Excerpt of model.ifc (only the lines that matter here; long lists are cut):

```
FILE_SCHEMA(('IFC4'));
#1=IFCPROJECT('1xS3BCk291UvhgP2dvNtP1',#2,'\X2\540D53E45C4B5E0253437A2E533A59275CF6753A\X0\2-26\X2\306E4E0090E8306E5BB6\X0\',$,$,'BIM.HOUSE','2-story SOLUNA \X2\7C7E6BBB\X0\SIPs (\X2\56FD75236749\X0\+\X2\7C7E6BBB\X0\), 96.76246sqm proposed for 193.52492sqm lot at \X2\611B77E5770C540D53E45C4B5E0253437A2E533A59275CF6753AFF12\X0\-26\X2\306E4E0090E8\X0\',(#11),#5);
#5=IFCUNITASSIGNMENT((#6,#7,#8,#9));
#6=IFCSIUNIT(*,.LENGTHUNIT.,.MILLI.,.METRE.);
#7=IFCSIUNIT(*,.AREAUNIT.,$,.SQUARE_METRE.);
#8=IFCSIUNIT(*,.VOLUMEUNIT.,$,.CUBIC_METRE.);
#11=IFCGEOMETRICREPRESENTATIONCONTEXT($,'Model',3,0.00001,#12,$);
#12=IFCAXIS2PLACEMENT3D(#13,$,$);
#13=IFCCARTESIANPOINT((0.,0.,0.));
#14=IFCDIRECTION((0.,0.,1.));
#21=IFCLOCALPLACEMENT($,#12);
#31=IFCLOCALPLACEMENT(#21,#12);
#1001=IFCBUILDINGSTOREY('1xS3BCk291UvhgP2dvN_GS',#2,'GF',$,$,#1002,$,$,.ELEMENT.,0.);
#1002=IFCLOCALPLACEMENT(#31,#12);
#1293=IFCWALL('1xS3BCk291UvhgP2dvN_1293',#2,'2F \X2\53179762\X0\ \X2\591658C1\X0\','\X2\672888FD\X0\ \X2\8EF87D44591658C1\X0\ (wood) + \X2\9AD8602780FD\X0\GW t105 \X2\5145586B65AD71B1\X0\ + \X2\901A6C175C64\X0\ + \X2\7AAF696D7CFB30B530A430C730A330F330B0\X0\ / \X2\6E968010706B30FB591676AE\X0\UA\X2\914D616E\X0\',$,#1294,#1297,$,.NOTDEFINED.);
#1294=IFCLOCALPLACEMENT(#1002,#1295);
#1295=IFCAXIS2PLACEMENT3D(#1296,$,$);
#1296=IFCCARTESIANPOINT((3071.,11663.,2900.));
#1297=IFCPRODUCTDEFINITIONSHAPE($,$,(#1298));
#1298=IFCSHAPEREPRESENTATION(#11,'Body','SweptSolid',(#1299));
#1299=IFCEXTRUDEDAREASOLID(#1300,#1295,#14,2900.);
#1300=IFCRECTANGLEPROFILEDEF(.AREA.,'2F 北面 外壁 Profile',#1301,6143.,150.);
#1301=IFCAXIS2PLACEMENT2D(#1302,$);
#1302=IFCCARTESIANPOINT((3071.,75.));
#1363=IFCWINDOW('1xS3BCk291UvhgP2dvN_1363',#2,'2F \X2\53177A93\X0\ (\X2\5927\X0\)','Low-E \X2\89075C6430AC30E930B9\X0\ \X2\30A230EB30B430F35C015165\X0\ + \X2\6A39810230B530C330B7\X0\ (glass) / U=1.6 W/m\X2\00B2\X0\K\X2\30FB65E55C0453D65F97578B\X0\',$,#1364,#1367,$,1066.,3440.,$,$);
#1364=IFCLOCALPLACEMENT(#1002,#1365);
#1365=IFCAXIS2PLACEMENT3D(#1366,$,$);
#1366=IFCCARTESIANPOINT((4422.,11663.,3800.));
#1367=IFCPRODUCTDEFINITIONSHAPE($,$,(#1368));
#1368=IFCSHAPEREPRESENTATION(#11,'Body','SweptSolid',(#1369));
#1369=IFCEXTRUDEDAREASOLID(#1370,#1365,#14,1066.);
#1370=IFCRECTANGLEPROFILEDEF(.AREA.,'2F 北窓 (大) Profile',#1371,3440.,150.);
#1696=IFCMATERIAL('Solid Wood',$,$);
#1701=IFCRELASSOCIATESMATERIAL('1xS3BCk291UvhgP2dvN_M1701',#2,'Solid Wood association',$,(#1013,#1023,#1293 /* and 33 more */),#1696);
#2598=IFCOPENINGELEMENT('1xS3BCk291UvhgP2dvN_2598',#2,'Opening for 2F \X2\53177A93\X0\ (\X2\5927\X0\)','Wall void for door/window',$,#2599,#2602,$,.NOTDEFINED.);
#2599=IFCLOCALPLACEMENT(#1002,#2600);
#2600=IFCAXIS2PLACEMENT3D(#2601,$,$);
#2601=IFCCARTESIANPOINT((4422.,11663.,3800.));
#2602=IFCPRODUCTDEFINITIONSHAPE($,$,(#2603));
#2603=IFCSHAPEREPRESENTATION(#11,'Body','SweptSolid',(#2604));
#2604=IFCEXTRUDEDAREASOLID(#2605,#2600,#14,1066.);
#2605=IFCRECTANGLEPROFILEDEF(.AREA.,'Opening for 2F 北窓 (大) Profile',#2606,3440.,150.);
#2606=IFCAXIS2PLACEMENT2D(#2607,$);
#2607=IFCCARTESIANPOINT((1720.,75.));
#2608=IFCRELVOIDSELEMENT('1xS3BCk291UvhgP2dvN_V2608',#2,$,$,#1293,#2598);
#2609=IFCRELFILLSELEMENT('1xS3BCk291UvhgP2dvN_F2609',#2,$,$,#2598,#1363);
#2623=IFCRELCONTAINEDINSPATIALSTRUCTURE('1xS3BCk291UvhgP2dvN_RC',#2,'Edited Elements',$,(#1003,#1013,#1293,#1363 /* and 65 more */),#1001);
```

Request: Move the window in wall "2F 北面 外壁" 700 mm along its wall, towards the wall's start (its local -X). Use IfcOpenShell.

```python
import ifcopenshell
import ifcopenshell.api.geometry
import ifcopenshell.util.placement

model = ifcopenshell.open("model.ifc")

window = model.by_guid("1xS3BCk291UvhgP2dvN_1363")
opening = window.FillsVoids[0].RelatingOpeningElement
wall = opening.VoidsElements[0].RelatingBuildingElement

wall_matrix = ifcopenshell.util.placement.get_local_placement(wall.ObjectPlacement)
shift = wall_matrix[:3, 0] * -700.0
before = ifcopenshell.util.placement.get_local_placement(window.ObjectPlacement)[:3, 3].copy()

# The window is not placed relative to its opening, so move both.
for product in (opening, window):
    matrix = ifcopenshell.util.placement.get_local_placement(product.ObjectPlacement)
    matrix[:3, 3] += shift
    ifcopenshell.api.geometry.edit_object_placement(model, product=product, matrix=matrix, is_si=False)

after = ifcopenshell.util.placement.get_local_placement(window.ObjectPlacement)[:3, 3]
print("window moved by", (after - before).round(3) + 0.0)

model.write("model_edited.ifc")
```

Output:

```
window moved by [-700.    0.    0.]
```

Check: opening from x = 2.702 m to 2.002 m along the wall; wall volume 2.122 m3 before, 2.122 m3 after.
